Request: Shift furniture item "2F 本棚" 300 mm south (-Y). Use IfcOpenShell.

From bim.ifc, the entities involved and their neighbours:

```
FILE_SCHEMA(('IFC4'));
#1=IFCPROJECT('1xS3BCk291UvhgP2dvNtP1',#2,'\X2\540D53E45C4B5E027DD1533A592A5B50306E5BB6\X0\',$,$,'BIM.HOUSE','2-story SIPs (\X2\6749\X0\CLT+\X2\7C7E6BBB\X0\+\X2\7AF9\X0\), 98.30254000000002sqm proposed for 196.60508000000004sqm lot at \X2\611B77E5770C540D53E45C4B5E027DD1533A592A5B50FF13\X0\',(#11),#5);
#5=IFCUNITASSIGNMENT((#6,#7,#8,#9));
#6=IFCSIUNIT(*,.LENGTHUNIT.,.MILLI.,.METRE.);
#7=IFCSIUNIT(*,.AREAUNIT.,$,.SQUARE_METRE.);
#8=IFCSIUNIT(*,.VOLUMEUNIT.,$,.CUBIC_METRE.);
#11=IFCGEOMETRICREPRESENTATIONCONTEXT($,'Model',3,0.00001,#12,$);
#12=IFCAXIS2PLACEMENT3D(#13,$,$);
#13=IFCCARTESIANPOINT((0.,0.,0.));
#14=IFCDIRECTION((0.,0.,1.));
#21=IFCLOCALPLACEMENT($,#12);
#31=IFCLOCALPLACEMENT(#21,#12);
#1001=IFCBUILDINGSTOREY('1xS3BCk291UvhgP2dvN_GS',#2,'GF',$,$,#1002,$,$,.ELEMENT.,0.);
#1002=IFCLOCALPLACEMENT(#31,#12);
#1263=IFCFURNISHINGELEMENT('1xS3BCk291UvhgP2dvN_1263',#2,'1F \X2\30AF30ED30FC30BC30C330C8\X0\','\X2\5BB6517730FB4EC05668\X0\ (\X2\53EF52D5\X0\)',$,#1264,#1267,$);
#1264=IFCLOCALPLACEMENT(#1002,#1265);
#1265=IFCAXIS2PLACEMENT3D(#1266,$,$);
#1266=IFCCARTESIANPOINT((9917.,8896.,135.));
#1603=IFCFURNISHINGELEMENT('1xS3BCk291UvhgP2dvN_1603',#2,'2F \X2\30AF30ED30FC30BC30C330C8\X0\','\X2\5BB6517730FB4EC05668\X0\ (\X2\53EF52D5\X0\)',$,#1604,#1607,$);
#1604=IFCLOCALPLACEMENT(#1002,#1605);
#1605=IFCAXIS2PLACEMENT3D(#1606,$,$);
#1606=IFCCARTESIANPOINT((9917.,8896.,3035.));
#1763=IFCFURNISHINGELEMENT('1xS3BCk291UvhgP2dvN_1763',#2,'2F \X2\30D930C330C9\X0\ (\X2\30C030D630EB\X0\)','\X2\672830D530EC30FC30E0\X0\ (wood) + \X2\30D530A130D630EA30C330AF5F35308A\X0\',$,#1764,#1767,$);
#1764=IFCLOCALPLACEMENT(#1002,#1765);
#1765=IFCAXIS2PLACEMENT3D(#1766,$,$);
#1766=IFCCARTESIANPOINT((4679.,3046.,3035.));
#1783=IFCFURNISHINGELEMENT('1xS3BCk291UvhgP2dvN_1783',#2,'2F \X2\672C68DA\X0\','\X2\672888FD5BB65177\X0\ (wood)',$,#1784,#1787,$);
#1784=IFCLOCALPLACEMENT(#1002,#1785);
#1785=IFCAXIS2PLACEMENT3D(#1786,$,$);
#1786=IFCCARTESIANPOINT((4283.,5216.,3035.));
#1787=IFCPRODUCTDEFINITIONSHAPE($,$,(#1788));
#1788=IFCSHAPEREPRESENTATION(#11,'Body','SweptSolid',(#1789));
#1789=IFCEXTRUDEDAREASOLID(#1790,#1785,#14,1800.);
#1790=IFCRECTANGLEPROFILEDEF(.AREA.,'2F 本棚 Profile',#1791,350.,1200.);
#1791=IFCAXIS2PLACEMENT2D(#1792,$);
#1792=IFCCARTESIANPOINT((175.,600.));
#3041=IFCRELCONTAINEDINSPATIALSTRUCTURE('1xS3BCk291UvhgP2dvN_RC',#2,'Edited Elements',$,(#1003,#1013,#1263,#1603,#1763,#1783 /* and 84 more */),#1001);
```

```python
import ifcopenshell
import ifcopenshell.api.geometry
import ifcopenshell.util.placement
import ifcopenshell.util.unit

model = ifcopenshell.open("bim.ifc")
unit_scale = ifcopenshell.util.unit.calculate_unit_scale(model)

item = model.by_guid("1xS3BCk291UvhgP2dvN_1783")
matrix = ifcopenshell.util.placement.get_local_placement(item.ObjectPlacement)
matrix[1, 3] -= 0.3 / unit_scale
ifcopenshell.api.geometry.edit_object_placement(model, product=item, matrix=matrix, is_si=False)

print(ifcopenshell.util.placement.get_local_placement(item.ObjectPlacement).round(3) + 0.0)

model.write("bim_updated.ifc")
```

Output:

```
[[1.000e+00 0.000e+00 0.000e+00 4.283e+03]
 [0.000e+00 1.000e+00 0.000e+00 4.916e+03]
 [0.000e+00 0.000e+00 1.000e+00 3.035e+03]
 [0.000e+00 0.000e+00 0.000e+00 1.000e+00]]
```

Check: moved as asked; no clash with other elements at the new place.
